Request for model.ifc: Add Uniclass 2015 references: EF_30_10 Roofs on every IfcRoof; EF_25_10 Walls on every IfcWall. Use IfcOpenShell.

First a look at what the model holds.

```python
import ifcopenshell

model = ifcopenshell.open("model.ifc")
print(model.schema)
print("classifications:", [c.Name for c in model.by_type("IfcClassification")])
for ifc_class in ("IfcDoor", "IfcRoof", "IfcStair", "IfcWall", "IfcWindow"):
    print(ifc_class, len(model.by_type(ifc_class)))
```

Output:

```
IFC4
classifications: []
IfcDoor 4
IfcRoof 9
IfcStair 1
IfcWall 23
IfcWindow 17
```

```python
import ifcopenshell
import ifcopenshell.api.classification

model = ifcopenshell.open("model.ifc")

system = ifcopenshell.api.classification.add_classification(model, classification="Uniclass 2015")

codes = {
    "IfcRoof": ("EF_30_10", "Roofs"),
    "IfcWall": ("EF_25_10", "Walls"),
}
for ifc_class, (code, name) in codes.items():
    products = model.by_type(ifc_class)
    ifcopenshell.api.classification.add_reference(
        model, products=products, classification=system, identification=code, name=name
    )
    print(code, len(products))

model.write("model_rev.ifc")
```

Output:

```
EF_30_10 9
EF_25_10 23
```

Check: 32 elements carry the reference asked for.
